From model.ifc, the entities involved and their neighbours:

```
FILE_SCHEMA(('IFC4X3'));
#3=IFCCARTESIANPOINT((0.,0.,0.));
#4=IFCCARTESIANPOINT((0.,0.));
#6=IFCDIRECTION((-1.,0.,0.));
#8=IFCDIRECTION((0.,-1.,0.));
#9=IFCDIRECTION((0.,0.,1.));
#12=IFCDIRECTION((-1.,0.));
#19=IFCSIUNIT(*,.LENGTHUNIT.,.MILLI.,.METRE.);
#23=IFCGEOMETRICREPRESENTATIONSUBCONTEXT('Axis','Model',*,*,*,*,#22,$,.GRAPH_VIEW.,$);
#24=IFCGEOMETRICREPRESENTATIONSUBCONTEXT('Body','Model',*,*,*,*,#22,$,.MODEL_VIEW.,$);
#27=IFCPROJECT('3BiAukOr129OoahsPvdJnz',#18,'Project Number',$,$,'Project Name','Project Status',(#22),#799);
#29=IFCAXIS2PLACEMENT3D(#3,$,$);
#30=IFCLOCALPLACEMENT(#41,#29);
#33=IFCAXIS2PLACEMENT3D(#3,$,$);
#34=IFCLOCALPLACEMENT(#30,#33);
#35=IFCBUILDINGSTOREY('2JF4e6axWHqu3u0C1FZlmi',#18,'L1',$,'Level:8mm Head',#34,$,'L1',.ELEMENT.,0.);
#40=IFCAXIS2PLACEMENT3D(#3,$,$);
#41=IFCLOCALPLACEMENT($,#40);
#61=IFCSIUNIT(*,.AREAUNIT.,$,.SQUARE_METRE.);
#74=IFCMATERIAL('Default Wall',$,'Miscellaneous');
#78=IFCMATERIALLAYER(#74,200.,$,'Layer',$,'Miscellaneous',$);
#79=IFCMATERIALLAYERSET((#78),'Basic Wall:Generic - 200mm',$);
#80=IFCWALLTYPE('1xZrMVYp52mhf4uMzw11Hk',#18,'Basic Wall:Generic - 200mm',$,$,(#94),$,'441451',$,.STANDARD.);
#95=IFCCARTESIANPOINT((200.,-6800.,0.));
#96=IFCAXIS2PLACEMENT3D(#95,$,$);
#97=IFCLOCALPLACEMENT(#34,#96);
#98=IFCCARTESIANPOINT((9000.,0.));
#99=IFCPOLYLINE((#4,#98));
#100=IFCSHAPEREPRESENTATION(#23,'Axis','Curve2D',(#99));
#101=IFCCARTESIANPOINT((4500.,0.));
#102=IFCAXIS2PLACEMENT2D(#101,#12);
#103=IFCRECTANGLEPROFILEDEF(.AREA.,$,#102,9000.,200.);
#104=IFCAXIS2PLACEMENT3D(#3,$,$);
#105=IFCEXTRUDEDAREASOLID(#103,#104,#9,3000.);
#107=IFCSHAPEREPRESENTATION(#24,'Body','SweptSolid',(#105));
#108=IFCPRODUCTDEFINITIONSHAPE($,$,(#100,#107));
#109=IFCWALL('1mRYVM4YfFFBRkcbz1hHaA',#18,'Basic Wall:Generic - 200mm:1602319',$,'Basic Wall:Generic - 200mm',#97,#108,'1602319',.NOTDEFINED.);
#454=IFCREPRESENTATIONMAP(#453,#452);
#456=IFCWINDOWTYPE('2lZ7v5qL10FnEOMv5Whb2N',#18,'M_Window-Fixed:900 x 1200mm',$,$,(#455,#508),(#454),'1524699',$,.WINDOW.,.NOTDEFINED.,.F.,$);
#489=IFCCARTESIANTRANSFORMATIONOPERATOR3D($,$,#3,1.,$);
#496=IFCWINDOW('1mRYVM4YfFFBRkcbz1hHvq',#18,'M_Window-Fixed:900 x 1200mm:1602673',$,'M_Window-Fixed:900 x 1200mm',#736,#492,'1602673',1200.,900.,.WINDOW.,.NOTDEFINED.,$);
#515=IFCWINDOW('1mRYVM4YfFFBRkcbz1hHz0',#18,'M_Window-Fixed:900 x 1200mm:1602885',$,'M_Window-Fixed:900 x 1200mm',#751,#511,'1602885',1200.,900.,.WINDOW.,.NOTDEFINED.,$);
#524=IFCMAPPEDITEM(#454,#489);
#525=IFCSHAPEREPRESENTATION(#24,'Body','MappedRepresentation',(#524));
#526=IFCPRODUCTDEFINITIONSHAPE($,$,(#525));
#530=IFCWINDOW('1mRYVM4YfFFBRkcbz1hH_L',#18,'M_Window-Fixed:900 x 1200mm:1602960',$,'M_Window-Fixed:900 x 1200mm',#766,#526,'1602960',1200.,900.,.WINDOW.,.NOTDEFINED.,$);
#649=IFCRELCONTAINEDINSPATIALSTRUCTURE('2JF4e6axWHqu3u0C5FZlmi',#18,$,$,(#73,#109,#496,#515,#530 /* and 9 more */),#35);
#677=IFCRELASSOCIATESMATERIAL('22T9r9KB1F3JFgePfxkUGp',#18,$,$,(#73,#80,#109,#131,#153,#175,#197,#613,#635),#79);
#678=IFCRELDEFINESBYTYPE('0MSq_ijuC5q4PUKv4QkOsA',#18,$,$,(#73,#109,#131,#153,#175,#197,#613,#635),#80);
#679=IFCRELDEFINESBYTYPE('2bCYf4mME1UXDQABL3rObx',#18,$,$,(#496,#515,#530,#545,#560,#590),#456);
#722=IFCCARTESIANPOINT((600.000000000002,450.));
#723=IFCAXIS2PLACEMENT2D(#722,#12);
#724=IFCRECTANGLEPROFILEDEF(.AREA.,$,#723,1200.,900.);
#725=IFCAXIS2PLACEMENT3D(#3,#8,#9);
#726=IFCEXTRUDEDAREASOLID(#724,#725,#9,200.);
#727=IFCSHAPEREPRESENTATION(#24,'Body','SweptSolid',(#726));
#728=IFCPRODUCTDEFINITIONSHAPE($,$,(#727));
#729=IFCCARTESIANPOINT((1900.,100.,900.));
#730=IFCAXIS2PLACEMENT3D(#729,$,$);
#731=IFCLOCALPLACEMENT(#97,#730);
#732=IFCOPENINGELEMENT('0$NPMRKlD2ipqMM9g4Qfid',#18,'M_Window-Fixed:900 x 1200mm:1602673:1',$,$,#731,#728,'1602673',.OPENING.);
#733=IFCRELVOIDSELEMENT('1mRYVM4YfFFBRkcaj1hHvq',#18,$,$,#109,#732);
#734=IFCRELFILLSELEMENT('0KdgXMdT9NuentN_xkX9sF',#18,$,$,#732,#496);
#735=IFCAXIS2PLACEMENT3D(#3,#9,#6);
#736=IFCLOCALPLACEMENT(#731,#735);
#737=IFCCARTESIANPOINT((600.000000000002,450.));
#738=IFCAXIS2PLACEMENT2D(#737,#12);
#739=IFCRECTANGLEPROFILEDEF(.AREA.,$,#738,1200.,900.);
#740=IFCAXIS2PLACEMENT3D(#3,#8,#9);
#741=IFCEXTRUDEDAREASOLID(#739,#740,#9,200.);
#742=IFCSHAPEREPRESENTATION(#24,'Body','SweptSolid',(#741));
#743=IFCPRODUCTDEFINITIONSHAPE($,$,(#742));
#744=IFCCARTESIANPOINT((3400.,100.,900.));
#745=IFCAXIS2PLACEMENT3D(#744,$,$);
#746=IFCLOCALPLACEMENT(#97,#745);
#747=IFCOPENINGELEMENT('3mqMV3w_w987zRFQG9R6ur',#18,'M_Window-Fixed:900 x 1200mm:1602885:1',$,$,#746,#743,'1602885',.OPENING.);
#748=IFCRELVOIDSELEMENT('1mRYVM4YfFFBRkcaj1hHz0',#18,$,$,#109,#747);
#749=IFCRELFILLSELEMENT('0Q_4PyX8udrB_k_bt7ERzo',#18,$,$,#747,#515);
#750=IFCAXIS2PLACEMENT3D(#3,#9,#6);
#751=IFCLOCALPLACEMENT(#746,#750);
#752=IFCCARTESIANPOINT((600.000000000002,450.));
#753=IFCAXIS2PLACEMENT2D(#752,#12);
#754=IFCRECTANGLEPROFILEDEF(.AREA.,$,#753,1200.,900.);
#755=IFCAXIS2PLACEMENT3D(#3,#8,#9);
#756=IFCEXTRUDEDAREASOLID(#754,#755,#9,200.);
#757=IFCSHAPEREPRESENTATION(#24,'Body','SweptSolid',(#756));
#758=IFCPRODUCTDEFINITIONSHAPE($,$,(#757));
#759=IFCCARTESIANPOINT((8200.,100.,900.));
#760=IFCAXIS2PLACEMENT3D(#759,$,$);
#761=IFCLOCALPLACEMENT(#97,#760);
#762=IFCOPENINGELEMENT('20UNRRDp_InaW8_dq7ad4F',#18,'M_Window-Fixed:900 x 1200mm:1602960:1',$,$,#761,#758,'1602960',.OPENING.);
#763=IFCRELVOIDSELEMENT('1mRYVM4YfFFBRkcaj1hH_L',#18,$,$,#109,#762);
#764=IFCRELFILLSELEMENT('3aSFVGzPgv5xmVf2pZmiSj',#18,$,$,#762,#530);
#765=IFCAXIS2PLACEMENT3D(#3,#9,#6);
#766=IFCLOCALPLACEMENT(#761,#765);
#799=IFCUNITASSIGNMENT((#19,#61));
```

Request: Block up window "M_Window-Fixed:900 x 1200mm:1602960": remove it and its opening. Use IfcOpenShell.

```python
import ifcopenshell
import ifcopenshell.api.feature
import ifcopenshell.api.root
import ifcopenshell.geom
import ifcopenshell.util.shape

model = ifcopenshell.open("model.ifc")
settings = ifcopenshell.geom.settings()


def volume(element):
    """Net volume in cubic metres, openings subtracted."""
    shape = ifcopenshell.geom.create_shape(settings, element)
    return ifcopenshell.util.shape.get_volume(shape.geometry)


window = model.by_guid("1mRYVM4YfFFBRkcbz1hH_L")
opening = window.FillsVoids[0].RelatingOpeningElement
wall = opening.VoidsElements[0].RelatingBuildingElement
before = volume(wall)

ifcopenshell.api.root.remove_product(model, product=window)
ifcopenshell.api.feature.remove_feature(model, feature=opening)

after = volume(wall)

print(f"wall volume {before:.3f} -> {after:.3f} m3")

model.write("model_v2.ifc")
```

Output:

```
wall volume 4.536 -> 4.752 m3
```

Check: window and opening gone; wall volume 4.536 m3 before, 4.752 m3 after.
